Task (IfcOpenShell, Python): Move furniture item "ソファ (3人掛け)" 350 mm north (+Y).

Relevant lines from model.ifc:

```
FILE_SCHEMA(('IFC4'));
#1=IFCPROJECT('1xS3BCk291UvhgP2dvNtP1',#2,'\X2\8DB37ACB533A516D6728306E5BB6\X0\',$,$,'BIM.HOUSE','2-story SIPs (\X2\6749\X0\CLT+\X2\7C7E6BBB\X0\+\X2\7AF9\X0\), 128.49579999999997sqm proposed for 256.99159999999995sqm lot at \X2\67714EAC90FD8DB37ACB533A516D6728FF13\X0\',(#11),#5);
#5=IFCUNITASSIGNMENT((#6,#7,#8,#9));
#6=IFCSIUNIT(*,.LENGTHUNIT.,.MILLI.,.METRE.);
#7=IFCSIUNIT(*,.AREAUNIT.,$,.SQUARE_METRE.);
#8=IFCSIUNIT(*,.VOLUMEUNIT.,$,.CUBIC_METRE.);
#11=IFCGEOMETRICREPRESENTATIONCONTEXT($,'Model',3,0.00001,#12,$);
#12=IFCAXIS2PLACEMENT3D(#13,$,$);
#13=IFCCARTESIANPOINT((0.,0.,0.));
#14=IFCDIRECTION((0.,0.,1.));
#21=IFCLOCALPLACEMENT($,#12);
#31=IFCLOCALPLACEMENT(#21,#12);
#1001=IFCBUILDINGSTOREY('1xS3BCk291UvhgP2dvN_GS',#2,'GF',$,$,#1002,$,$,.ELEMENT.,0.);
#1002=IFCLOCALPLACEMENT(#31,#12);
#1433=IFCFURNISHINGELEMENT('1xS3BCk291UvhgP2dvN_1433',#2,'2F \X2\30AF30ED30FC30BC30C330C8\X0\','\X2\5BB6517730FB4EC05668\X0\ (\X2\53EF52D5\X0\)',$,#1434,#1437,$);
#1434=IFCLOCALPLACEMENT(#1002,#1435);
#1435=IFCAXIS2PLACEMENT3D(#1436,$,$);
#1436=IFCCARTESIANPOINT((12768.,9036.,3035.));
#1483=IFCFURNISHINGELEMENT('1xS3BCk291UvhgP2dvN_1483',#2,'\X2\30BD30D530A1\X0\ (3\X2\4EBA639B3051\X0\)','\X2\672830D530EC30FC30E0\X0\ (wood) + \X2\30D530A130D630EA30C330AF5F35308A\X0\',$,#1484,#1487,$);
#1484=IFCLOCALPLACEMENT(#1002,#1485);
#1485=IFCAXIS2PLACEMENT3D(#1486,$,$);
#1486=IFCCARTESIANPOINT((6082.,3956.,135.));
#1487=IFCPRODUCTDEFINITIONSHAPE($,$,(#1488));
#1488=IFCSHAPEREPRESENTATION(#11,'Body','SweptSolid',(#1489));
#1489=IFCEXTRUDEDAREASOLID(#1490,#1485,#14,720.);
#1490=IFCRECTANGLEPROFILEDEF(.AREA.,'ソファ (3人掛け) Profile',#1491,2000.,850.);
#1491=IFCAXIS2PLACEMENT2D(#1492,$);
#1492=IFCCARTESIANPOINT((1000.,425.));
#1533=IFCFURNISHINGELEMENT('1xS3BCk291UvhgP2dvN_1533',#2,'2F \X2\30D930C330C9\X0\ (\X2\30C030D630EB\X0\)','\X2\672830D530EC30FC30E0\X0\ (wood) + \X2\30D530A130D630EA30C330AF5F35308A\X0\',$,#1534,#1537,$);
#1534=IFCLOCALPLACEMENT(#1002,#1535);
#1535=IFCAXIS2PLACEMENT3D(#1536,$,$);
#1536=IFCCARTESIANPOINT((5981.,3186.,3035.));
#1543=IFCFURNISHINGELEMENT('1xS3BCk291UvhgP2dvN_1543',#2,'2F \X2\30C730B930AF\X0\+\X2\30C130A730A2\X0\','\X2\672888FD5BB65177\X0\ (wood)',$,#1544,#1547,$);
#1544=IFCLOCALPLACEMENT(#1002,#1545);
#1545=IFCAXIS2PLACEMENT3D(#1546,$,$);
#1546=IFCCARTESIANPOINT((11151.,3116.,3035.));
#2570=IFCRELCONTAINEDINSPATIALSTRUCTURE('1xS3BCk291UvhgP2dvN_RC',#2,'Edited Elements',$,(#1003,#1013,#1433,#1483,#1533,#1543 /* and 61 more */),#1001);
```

```python
import ifcopenshell
import ifcopenshell.api.geometry
import ifcopenshell.util.placement
import ifcopenshell.util.unit

model = ifcopenshell.open("model.ifc")
unit_scale = ifcopenshell.util.unit.calculate_unit_scale(model)

item = model.by_id(1483)
matrix = ifcopenshell.util.placement.get_local_placement(item.ObjectPlacement)
matrix[1, 3] += 0.35 / unit_scale
ifcopenshell.api.geometry.edit_object_placement(model, product=item, matrix=matrix, is_si=False)

print(ifcopenshell.util.placement.get_local_placement(item.ObjectPlacement).round(3) + 0.0)

model.write("model_updated.ifc")
```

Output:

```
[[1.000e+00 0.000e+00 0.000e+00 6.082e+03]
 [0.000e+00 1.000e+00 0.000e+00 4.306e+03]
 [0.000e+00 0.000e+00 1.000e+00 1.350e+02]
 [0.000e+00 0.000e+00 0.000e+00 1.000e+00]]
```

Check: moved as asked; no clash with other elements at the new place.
